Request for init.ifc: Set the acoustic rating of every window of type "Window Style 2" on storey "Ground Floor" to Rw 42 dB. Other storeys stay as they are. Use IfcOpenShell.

First a look at what the model holds.

```python
import ifcopenshell
import ifcopenshell.util.element

model = ifcopenshell.open("init.ifc")
print(model.schema)
storey = next(s for s in model.by_type("IfcBuildingStorey") if s.Name == "Ground Floor")
windows = [e for e in ifcopenshell.util.element.get_decomposition(storey) if e.is_a("IfcWindow")]
seen = {}
for e in windows:
    element_type = ifcopenshell.util.element.get_type(e)
    key = (element_type.Name if element_type != e and element_type else None, ifcopenshell.util.element.get_pset(e, "Pset_WindowCommon", "AcousticRating"))
    seen[key] = seen.get(key, 0) + 1
for (name, value), count in sorted(seen.items(), key=str):
    print(count, "x", name, "|", value)
```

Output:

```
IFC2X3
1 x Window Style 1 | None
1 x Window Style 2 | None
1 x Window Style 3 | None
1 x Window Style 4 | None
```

```python
import ifcopenshell
import ifcopenshell.api.pset
import ifcopenshell.util.element

model = ifcopenshell.open("init.ifc")

storey = next(s for s in model.by_type("IfcBuildingStorey") if s.Name == "Ground Floor")
windows = [e for e in ifcopenshell.util.element.get_decomposition(storey) if e.is_a("IfcWindow")]

count = 0
for e in windows:
    element_type = ifcopenshell.util.element.get_type(e)
    if element_type in (None, e) or element_type.Name != "Window Style 2":
        continue
    # add_pset returns the element's existing set when there is one.
    pset = ifcopenshell.api.pset.add_pset(model, product=e, name="Pset_WindowCommon")
    ifcopenshell.api.pset.edit_pset(model, pset=pset, properties={"AcousticRating": "Rw 42 dB"})
    count += 1

print(count, "windows updated")

model.write("init-out.ifc")
```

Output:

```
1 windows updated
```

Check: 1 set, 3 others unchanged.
